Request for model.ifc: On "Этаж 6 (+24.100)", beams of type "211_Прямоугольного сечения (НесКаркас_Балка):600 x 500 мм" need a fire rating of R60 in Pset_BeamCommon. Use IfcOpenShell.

First a look at what the model holds.

```python
import ifcopenshell
import ifcopenshell.util.element

model = ifcopenshell.open("model.ifc")
print(model.schema)
storey = next(s for s in model.by_type("IfcBuildingStorey") if s.Name == "Этаж 6 (+24.100)")
beams = [e for e in ifcopenshell.util.element.get_decomposition(storey) if e.is_a("IfcBeam")]
seen = {}
for e in beams:
    element_type = ifcopenshell.util.element.get_type(e)
    key = (element_type.Name if element_type != e and element_type else None, ifcopenshell.util.element.get_pset(e, "Pset_BeamCommon", "FireRating"))
    seen[key] = seen.get(key, 0) + 1
for (name, value), count in sorted(seen.items(), key=str):
    print(count, "x", name, "|", value)
```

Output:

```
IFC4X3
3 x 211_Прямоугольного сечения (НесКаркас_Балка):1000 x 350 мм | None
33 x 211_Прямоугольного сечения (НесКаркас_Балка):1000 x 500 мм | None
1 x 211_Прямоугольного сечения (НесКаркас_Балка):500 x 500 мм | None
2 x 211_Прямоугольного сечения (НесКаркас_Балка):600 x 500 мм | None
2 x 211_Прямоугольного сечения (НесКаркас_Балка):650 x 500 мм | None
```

```python
import ifcopenshell
import ifcopenshell.api.pset
import ifcopenshell.util.element

model = ifcopenshell.open("model.ifc")

storey = next(s for s in model.by_type("IfcBuildingStorey") if s.Name == "Этаж 6 (+24.100)")
beams = [e for e in ifcopenshell.util.element.get_decomposition(storey) if e.is_a("IfcBeam")]

count = 0
for e in beams:
    element_type = ifcopenshell.util.element.get_type(e)
    if element_type in (None, e) or element_type.Name != "211_Прямоугольного сечения (НесКаркас_Балка):600 x 500 мм":
        continue
    # add_pset returns the element's existing set when there is one.
    pset = ifcopenshell.api.pset.add_pset(model, product=e, name="Pset_BeamCommon")
    ifcopenshell.api.pset.edit_pset(model, pset=pset, properties={"FireRating": "R60"})
    count += 1

print(count, "beams updated")

model.write("model_updated.ifc")
```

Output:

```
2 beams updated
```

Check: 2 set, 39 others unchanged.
